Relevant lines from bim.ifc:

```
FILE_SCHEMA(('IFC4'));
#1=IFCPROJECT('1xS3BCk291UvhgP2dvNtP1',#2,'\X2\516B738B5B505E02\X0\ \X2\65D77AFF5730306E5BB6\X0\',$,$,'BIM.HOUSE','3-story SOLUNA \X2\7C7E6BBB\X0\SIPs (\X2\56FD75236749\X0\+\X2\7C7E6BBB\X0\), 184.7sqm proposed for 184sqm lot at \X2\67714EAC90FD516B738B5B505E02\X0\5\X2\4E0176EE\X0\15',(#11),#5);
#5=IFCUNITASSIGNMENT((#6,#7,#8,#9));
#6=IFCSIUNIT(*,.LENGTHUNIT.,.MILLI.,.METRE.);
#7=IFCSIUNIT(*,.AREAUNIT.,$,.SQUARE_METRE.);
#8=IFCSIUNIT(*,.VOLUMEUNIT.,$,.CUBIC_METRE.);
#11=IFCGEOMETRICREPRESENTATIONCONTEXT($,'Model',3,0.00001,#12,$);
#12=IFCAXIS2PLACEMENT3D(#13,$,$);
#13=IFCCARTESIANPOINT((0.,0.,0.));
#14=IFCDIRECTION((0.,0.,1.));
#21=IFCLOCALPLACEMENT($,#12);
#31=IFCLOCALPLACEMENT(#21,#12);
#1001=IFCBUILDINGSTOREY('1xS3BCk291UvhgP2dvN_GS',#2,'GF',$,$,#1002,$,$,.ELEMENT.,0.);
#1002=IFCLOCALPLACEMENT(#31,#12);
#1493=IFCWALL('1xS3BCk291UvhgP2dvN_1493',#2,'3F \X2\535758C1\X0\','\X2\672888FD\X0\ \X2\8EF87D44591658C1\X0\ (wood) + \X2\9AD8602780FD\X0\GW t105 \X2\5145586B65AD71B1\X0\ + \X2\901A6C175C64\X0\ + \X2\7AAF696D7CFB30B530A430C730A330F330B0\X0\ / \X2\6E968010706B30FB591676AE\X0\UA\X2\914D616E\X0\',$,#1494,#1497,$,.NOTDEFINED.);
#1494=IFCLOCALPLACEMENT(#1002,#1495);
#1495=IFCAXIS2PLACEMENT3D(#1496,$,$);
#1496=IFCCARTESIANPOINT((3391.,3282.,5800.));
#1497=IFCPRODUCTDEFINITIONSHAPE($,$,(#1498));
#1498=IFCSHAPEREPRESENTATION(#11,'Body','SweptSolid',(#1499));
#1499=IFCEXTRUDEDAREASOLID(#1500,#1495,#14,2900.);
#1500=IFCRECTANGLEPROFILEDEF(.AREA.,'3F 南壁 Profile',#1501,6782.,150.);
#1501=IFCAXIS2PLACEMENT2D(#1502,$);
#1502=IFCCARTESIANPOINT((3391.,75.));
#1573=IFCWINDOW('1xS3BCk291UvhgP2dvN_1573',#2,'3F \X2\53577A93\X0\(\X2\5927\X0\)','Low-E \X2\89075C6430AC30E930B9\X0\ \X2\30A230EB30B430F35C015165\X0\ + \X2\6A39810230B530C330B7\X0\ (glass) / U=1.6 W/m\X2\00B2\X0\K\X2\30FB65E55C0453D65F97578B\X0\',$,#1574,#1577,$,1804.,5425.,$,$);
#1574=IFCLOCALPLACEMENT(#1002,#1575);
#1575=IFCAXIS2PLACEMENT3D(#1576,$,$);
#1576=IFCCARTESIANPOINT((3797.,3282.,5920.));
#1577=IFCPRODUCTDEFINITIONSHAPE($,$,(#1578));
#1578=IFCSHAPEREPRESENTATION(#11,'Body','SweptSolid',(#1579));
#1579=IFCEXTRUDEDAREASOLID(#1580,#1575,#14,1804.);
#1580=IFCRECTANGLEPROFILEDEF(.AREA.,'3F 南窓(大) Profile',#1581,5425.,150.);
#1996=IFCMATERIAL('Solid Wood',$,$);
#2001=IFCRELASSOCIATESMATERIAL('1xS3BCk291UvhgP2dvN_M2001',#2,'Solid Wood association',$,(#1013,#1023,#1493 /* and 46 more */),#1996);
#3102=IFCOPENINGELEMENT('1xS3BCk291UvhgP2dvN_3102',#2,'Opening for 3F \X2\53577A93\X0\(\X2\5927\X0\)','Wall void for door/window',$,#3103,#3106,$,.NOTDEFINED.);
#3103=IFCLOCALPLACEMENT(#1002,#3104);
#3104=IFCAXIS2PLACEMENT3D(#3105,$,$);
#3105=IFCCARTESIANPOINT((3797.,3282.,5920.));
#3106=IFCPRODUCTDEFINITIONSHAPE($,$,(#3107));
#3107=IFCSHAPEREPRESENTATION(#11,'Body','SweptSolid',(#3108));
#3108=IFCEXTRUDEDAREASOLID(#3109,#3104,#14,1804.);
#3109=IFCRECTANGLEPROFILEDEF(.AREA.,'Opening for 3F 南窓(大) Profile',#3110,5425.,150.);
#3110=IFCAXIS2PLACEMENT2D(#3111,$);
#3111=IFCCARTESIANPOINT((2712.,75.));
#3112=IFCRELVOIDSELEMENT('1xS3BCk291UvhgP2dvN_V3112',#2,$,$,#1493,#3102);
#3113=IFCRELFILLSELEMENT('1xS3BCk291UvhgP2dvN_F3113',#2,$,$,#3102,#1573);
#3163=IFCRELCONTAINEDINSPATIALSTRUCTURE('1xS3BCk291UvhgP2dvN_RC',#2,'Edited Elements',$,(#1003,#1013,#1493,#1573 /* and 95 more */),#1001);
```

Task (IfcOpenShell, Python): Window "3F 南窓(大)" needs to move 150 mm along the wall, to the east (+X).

```python
import ifcopenshell
import ifcopenshell.api.geometry
import ifcopenshell.util.placement
import ifcopenshell.util.unit

model = ifcopenshell.open("bim.ifc")
unit_scale = ifcopenshell.util.unit.calculate_unit_scale(model)

window = model.by_guid("1xS3BCk291UvhgP2dvN_1573")
opening = window.FillsVoids[0].RelatingOpeningElement
wall = opening.VoidsElements[0].RelatingBuildingElement

wall_matrix = ifcopenshell.util.placement.get_local_placement(wall.ObjectPlacement)
shift = wall_matrix[:3, 0] * 0.15 / unit_scale
before = ifcopenshell.util.placement.get_local_placement(window.ObjectPlacement)[:3, 3].copy()

# The window is not placed relative to its opening, so move both.
for product in (opening, window):
    matrix = ifcopenshell.util.placement.get_local_placement(product.ObjectPlacement)
    matrix[:3, 3] += shift
    ifcopenshell.api.geometry.edit_object_placement(model, product=product, matrix=matrix, is_si=False)

after = ifcopenshell.util.placement.get_local_placement(window.ObjectPlacement)[:3, 3]
print("window moved by", (after - before).round(3) + 0.0)

model.write("bim_updated.ifc")
```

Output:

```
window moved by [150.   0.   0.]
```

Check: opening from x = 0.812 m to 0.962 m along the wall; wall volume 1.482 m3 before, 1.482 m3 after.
